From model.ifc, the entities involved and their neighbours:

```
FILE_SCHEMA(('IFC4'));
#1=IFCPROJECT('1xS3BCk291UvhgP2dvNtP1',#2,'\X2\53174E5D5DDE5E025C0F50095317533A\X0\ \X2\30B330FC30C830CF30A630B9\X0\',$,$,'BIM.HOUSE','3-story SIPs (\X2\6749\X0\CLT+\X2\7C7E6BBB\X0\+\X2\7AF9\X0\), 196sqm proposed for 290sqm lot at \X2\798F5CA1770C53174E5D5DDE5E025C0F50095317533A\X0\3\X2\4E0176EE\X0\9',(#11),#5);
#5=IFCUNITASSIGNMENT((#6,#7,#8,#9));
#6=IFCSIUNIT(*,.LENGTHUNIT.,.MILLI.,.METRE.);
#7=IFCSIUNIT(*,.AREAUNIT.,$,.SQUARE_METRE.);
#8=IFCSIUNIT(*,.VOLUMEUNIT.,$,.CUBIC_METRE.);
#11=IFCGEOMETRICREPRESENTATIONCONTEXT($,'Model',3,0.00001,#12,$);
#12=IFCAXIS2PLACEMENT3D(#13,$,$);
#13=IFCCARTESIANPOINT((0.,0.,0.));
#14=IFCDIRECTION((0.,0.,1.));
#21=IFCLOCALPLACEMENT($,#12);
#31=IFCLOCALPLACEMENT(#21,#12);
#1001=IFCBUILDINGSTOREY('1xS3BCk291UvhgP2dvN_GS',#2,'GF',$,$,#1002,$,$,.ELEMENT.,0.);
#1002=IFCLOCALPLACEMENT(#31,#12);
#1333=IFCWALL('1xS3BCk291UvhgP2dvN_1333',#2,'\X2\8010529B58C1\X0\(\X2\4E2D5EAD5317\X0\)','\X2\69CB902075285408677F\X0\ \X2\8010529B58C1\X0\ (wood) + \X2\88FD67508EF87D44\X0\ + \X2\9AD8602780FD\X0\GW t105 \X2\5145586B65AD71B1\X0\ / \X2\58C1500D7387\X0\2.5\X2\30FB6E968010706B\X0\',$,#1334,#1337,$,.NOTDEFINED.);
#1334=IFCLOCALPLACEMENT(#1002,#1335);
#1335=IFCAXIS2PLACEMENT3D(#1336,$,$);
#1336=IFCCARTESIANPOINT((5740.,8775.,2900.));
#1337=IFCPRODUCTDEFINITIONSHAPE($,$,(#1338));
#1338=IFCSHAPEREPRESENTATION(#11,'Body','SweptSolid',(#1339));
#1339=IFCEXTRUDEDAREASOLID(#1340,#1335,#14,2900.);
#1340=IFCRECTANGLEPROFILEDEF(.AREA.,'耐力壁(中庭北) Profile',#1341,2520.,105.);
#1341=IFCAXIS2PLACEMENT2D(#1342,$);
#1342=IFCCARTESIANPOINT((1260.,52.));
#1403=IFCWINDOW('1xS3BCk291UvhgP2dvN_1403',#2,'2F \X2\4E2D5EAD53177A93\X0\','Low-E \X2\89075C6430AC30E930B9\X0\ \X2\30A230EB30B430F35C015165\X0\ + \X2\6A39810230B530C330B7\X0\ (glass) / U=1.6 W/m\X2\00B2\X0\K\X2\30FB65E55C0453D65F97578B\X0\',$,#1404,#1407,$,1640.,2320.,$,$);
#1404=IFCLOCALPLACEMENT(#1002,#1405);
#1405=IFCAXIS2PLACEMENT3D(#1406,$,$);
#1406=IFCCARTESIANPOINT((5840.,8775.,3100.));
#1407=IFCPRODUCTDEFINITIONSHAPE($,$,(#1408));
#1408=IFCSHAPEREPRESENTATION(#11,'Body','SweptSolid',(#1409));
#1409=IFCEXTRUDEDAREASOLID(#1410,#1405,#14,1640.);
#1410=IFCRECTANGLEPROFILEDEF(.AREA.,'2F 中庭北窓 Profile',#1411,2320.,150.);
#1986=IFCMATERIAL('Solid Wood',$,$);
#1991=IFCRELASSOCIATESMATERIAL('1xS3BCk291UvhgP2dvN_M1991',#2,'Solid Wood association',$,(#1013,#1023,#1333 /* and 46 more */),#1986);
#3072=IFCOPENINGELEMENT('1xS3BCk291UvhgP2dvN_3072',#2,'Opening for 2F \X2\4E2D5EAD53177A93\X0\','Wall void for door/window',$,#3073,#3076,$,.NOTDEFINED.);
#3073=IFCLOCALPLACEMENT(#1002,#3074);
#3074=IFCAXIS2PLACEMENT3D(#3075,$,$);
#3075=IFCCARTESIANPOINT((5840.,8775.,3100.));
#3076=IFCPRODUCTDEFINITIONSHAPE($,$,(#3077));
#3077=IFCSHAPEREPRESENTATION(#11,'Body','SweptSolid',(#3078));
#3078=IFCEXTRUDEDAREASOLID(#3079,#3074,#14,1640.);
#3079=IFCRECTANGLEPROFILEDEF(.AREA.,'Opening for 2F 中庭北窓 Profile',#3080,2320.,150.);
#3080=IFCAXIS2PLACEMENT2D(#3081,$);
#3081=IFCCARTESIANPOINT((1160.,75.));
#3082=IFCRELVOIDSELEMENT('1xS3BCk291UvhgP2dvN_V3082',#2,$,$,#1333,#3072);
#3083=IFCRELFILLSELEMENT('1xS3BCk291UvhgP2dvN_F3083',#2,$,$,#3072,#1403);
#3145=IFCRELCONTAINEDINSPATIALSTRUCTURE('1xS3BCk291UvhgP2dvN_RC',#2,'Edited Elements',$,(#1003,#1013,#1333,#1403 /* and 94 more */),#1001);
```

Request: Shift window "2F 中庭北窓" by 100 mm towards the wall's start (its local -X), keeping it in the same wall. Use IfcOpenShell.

```python
import ifcopenshell
import ifcopenshell.api.geometry
import ifcopenshell.util.placement

model = ifcopenshell.open("model.ifc")

window = model.by_id(1403)
opening = window.FillsVoids[0].RelatingOpeningElement
wall = opening.VoidsElements[0].RelatingBuildingElement

wall_matrix = ifcopenshell.util.placement.get_local_placement(wall.ObjectPlacement)
shift = wall_matrix[:3, 0] * -100.0
before = ifcopenshell.util.placement.get_local_placement(window.ObjectPlacement)[:3, 3].copy()

# The window is not placed relative to its opening, so move both.
for product in (opening, window):
    matrix = ifcopenshell.util.placement.get_local_placement(product.ObjectPlacement)
    matrix[:3, 3] += shift
    ifcopenshell.api.geometry.edit_object_placement(model, product=product, matrix=matrix, is_si=False)

after = ifcopenshell.util.placement.get_local_placement(window.ObjectPlacement)[:3, 3]
print("window moved by", (after - before).round(3) + 0.0)

model.write("model_v2.ifc")
```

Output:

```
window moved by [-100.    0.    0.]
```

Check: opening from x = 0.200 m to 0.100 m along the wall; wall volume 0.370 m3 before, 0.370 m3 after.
